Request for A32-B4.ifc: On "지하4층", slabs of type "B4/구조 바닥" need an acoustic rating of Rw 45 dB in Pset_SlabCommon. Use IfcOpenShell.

First a look at what the model holds.

```python
import ifcopenshell
import ifcopenshell.util.element

model = ifcopenshell.open("A32-B4.ifc")
print(model.schema)
storey = next(s for s in model.by_type("IfcBuildingStorey") if s.Name == "지하4층")
slabs = [e for e in ifcopenshell.util.element.get_decomposition(storey) if e.is_a("IfcSlab")]
seen = {}
for e in slabs:
    element_type = ifcopenshell.util.element.get_type(e)
    key = (element_type.Name if element_type != e and element_type else None, ifcopenshell.util.element.get_pset(e, "Pset_SlabCommon", "AcousticRating"))
    seen[key] = seen.get(key, 0) + 1
for (name, value), count in sorted(seen.items(), key=str):
    print(count, "x", name, "|", value)
```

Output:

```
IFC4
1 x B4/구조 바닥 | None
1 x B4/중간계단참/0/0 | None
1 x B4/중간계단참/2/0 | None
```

```python
import ifcopenshell
import ifcopenshell.api.pset
import ifcopenshell.util.element

model = ifcopenshell.open("A32-B4.ifc")

storey = next(s for s in model.by_type("IfcBuildingStorey") if s.Name == "지하4층")
slabs = [e for e in ifcopenshell.util.element.get_decomposition(storey) if e.is_a("IfcSlab")]

count = 0
for e in slabs:
    element_type = ifcopenshell.util.element.get_type(e)
    if element_type in (None, e) or element_type.Name != "B4/구조 바닥":
        continue
    # add_pset returns the element's existing set when there is one.
    pset = ifcopenshell.api.pset.add_pset(model, product=e, name="Pset_SlabCommon")
    ifcopenshell.api.pset.edit_pset(model, pset=pset, properties={"AcousticRating": "Rw 45 dB"})
    count += 1

print(count, "slabs updated")

model.write("A32-B4_edited.ifc")
```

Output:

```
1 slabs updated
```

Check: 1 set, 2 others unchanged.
